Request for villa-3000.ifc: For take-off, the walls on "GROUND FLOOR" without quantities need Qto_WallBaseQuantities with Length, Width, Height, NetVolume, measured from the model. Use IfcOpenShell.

First a look at what the model holds.

```python
import ifcopenshell
import ifcopenshell.util.element
import ifcopenshell.util.unit

model = ifcopenshell.open("villa-3000.ifc")
print(model.schema)
for unit_type in ("LENGTHUNIT", "AREAUNIT", "VOLUMEUNIT"):
    print(unit_type, ifcopenshell.util.unit.calculate_unit_scale(model, unit_type))
storey = next(s for s in model.by_type("IfcBuildingStorey") if s.Name == "GROUND FLOOR")
walls = [e for e in ifcopenshell.util.element.get_decomposition(storey) if e.is_a("IfcWall")]
for e in sorted(walls, key=lambda e: e.id()):
    print(e.id(), e.is_a(), e.Name, list(ifcopenshell.util.element.get_psets(e, qtos_only=True)), sep=" | ")
```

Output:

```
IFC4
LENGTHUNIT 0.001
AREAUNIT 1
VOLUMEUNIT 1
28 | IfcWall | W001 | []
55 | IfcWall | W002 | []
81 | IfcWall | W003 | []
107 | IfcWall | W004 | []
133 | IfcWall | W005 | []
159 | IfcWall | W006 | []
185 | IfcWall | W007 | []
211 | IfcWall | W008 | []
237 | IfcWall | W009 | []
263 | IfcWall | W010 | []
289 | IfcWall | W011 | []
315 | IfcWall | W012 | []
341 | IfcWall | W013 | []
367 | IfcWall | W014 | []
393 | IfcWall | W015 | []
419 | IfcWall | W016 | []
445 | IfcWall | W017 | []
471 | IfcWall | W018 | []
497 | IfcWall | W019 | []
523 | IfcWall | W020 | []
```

```python
import ifcopenshell
import ifcopenshell.api.pset
import ifcopenshell.geom
import ifcopenshell.util.element
import ifcopenshell.util.shape
import ifcopenshell.util.unit

model = ifcopenshell.open("villa-3000.ifc")
unit_scale = ifcopenshell.util.unit.calculate_unit_scale(model)
volume_scale = ifcopenshell.util.unit.calculate_unit_scale(model, "VOLUMEUNIT")
settings = ifcopenshell.geom.settings()

storey = next(s for s in model.by_type("IfcBuildingStorey") if s.Name == "GROUND FLOOR")
walls = [e for e in ifcopenshell.util.element.get_decomposition(storey) if e.is_a("IfcWall")]

for e in sorted(walls, key=lambda e: e.id()):
    if ifcopenshell.util.element.get_psets(e, qtos_only=True, should_inherit=False):
        continue
    # Geometry comes back in metres, in the element's own axes.
    shape = ifcopenshell.geom.create_shape(settings, e)
    values = {
        "Length": ifcopenshell.util.shape.get_x(shape.geometry) / unit_scale,
        "Width": ifcopenshell.util.shape.get_y(shape.geometry) / unit_scale,
        "Height": ifcopenshell.util.shape.get_z(shape.geometry) / unit_scale,
        "NetVolume": ifcopenshell.util.shape.get_volume(shape.geometry) / volume_scale,
    }
    qto = ifcopenshell.api.pset.add_qto(model, product=e, name="Qto_WallBaseQuantities")
    ifcopenshell.api.pset.edit_qto(model, qto=qto, properties=values)
    print(e.id(), {k: round(v, 3) for k, v in values.items()})

model.write("villa-3000_rev.ifc")
```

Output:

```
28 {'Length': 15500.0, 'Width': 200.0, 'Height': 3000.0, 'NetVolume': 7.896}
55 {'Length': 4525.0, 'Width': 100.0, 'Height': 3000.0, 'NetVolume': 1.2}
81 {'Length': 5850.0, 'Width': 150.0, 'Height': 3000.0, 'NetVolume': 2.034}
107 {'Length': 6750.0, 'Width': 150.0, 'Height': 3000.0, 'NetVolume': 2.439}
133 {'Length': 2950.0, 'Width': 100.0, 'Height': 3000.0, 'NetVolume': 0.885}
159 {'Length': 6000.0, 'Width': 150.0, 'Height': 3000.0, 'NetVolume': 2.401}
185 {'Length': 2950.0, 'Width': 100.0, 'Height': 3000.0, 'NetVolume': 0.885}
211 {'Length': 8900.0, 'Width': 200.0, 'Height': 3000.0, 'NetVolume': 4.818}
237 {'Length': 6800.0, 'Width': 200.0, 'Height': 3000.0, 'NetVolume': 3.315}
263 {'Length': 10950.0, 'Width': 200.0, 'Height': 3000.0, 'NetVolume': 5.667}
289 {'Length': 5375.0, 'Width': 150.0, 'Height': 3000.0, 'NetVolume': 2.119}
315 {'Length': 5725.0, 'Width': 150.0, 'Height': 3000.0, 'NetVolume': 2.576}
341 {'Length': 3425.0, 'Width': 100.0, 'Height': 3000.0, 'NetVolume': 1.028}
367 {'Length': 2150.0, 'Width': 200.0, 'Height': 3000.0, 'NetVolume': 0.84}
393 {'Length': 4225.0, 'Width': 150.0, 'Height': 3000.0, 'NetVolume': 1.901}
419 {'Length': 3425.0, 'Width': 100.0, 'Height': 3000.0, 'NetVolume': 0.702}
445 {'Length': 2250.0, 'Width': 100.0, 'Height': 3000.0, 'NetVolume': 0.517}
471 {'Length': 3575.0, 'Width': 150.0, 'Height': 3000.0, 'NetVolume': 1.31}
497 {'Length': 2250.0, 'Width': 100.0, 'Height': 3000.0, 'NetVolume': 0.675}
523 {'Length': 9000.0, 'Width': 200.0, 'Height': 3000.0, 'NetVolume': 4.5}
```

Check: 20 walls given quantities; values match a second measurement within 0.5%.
